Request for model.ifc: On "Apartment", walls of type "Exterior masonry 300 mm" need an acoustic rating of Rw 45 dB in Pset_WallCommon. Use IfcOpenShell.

First a look at what the model holds.

```python
import ifcopenshell
import ifcopenshell.util.element

model = ifcopenshell.open("model.ifc")
print(model.schema)
storey = next(s for s in model.by_type("IfcBuildingStorey") if s.Name == "Apartment")
walls = [e for e in ifcopenshell.util.element.get_decomposition(storey) if e.is_a("IfcWall")]
seen = {}
for e in walls:
    element_type = ifcopenshell.util.element.get_type(e)
    key = (element_type.Name if element_type != e and element_type else None, ifcopenshell.util.element.get_pset(e, "Pset_WallCommon", "AcousticRating"))
    seen[key] = seen.get(key, 0) + 1
for (name, value), count in sorted(seen.items(), key=str):
    print(count, "x", name, "|", value)
```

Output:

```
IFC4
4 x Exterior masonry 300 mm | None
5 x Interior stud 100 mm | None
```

```python
import ifcopenshell
import ifcopenshell.api.pset
import ifcopenshell.util.element

model = ifcopenshell.open("model.ifc")

storey = next(s for s in model.by_type("IfcBuildingStorey") if s.Name == "Apartment")
walls = [e for e in ifcopenshell.util.element.get_decomposition(storey) if e.is_a("IfcWall")]

count = 0
for e in walls:
    element_type = ifcopenshell.util.element.get_type(e)
    if element_type in (None, e) or element_type.Name != "Exterior masonry 300 mm":
        continue
    # add_pset returns the element's existing set when there is one.
    pset = ifcopenshell.api.pset.add_pset(model, product=e, name="Pset_WallCommon")
    ifcopenshell.api.pset.edit_pset(model, pset=pset, properties={"AcousticRating": "Rw 45 dB"})
    count += 1

print(count, "walls updated")

model.write("model_updated.ifc")
```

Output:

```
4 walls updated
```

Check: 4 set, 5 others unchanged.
